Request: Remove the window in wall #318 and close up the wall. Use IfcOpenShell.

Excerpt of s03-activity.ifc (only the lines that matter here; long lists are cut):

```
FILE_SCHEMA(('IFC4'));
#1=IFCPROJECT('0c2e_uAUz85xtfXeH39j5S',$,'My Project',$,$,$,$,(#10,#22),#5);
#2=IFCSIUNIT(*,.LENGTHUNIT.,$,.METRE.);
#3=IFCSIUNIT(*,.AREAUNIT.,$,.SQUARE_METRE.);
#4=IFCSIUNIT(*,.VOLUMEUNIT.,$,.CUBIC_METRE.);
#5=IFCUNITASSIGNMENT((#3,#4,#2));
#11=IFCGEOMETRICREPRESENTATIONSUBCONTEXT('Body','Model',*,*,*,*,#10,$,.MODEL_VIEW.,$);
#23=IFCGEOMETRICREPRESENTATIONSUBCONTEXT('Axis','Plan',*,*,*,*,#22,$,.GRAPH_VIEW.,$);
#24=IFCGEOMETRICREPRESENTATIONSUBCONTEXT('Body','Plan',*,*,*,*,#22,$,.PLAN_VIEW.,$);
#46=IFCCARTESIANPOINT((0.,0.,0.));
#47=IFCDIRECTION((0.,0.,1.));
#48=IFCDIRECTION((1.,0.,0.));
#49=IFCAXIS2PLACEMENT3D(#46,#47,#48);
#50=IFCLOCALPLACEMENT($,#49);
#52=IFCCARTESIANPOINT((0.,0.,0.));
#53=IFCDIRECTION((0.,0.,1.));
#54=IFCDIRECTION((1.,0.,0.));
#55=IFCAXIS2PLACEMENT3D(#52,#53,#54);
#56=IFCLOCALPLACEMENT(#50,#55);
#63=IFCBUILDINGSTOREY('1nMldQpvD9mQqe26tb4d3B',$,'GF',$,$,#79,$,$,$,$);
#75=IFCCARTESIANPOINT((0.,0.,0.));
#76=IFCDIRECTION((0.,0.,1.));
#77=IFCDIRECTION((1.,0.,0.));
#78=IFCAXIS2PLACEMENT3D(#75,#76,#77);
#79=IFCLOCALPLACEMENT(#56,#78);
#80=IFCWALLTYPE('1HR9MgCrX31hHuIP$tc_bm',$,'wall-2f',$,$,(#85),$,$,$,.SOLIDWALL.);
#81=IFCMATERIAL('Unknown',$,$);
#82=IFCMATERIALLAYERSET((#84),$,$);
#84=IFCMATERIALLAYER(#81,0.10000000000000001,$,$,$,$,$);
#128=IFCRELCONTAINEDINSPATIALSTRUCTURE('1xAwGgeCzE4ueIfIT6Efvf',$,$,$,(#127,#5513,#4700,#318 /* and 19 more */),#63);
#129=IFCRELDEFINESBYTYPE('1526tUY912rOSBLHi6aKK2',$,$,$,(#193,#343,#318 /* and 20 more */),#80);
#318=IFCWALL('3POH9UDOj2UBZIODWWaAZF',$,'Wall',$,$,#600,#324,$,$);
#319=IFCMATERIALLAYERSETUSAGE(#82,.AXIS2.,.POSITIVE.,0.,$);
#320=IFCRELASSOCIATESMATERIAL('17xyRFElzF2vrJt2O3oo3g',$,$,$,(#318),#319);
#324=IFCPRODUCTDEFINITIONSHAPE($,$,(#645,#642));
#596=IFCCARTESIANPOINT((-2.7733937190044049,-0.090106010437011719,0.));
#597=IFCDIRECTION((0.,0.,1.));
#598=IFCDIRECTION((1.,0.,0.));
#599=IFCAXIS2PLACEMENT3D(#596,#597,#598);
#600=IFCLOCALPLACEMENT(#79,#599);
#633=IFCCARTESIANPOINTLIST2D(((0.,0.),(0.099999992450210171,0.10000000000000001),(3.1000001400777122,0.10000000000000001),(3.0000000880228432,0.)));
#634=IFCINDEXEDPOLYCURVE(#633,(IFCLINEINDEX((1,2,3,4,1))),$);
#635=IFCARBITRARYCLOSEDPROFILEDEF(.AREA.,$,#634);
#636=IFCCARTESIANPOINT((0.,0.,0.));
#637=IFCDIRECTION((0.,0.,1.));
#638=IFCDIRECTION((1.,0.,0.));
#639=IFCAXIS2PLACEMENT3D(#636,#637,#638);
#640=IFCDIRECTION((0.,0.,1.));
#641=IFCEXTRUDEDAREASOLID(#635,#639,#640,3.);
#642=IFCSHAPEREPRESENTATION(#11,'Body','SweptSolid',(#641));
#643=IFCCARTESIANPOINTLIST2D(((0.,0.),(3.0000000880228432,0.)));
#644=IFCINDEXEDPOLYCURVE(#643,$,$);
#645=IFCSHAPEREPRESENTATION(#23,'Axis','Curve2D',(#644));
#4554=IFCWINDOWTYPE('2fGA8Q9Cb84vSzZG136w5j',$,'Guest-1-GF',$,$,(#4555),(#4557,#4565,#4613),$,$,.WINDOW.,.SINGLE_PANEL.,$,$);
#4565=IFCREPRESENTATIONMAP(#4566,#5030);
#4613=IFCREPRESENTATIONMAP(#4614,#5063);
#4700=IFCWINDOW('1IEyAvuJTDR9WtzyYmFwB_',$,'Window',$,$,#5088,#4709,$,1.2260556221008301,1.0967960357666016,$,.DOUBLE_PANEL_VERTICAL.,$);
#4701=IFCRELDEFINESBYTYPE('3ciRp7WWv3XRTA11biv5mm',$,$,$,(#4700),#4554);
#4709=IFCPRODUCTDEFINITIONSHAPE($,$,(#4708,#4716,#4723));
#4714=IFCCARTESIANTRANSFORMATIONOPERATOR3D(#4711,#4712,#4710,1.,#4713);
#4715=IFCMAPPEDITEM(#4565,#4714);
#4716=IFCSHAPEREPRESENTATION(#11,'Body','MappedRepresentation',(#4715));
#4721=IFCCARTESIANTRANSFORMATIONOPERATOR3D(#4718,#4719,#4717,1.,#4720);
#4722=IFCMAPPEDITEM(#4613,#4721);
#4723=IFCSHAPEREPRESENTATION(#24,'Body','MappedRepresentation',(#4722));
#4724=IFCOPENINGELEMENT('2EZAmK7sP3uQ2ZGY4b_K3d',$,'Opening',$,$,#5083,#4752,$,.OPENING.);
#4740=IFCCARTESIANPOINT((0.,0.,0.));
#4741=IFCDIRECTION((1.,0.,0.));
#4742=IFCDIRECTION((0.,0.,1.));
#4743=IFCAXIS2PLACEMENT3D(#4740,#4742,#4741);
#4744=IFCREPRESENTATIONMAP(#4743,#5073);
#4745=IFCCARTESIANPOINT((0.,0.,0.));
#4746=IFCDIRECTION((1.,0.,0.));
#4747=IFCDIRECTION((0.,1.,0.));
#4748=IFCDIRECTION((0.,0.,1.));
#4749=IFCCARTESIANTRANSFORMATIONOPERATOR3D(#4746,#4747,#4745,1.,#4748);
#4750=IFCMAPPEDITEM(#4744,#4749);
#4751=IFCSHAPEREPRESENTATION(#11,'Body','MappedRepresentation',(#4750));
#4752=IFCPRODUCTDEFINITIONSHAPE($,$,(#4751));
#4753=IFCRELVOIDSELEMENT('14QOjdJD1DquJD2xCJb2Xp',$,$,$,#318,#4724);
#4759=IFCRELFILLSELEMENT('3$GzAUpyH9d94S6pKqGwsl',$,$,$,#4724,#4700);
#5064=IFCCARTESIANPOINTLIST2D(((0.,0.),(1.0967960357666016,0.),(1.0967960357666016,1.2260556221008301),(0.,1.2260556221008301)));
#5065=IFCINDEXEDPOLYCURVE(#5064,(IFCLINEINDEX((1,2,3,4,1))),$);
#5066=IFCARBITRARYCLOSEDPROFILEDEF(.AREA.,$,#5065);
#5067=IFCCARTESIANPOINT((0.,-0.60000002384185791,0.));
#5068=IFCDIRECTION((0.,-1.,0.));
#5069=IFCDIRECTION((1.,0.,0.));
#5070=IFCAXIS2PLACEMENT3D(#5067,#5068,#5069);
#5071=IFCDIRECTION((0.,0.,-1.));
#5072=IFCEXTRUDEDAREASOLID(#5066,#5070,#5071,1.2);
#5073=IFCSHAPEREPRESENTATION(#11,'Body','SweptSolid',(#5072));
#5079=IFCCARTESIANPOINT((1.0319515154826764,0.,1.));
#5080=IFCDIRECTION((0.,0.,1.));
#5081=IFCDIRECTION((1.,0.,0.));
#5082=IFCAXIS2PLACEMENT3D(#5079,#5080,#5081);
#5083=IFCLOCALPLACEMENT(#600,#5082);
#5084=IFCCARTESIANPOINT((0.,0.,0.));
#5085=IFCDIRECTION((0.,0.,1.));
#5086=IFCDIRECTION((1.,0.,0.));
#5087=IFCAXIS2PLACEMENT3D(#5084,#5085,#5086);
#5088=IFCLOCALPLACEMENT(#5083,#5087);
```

```python
import ifcopenshell
import ifcopenshell.api.feature
import ifcopenshell.api.root
import ifcopenshell.geom
import ifcopenshell.util.shape

model = ifcopenshell.open("s03-activity.ifc")
settings = ifcopenshell.geom.settings()


def volume(element):
    """Net volume in cubic metres, openings subtracted."""
    shape = ifcopenshell.geom.create_shape(settings, element)
    return ifcopenshell.util.shape.get_volume(shape.geometry)


window = model.by_guid("1IEyAvuJTDR9WtzyYmFwB_")
opening = window.FillsVoids[0].RelatingOpeningElement
wall = opening.VoidsElements[0].RelatingBuildingElement
before = volume(wall)

ifcopenshell.api.root.remove_product(model, product=window)
ifcopenshell.api.feature.remove_feature(model, feature=opening)

after = volume(wall)

print(f"wall volume {before:.3f} -> {after:.3f} m3")

model.write("s03-activity_rev.ifc")
```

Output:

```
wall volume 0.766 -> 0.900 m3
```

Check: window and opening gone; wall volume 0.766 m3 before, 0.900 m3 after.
